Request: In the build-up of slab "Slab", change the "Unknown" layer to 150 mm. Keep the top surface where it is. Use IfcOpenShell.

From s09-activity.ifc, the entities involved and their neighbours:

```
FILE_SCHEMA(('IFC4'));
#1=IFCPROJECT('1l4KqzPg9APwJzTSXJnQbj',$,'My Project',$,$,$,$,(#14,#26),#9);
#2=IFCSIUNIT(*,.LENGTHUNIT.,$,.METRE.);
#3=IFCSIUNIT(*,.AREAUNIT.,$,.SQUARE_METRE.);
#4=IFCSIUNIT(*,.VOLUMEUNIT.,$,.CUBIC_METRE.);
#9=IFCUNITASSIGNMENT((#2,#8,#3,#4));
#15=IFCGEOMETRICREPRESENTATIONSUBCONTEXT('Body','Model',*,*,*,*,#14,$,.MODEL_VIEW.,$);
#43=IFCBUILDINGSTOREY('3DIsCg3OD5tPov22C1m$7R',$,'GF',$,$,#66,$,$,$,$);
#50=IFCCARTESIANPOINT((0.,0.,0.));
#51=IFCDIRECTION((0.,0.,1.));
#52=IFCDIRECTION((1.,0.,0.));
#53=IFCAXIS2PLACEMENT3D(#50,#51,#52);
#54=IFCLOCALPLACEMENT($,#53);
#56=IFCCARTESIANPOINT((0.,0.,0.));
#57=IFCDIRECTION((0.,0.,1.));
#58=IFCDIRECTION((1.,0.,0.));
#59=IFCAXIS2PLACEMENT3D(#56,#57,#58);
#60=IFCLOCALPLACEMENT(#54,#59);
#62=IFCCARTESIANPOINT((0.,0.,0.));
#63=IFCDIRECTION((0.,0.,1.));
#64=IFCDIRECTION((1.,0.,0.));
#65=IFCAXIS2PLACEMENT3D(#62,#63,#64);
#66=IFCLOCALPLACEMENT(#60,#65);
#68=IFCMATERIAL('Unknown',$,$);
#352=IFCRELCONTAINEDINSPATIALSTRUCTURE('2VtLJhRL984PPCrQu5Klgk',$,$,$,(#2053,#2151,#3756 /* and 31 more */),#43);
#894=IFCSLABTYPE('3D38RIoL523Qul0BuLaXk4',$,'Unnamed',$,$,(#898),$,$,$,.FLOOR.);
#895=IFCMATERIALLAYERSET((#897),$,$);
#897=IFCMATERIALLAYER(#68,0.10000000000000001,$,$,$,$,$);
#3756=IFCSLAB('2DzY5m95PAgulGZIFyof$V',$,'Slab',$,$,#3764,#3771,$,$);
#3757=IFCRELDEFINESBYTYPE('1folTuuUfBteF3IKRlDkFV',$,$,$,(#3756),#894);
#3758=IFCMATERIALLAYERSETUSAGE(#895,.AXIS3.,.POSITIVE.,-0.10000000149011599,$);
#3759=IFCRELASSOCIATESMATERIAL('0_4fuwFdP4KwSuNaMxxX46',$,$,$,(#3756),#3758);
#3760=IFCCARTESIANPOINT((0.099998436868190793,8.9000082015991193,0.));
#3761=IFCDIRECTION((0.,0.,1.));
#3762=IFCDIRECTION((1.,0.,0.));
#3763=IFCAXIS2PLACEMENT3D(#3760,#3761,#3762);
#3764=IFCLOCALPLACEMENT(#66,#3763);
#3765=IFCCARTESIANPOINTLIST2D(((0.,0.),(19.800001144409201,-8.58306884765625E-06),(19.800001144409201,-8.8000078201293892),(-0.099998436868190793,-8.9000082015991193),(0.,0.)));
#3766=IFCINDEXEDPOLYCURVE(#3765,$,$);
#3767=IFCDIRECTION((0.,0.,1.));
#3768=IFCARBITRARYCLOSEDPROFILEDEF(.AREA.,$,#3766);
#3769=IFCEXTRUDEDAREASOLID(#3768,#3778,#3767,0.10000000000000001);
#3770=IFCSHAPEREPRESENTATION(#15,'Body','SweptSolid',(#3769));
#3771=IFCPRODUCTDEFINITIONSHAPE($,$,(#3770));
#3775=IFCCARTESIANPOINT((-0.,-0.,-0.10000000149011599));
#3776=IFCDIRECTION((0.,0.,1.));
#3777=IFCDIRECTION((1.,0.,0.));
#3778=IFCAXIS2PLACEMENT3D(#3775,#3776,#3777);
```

```python
import ifcopenshell
import ifcopenshell.util.element
import ifcopenshell.util.representation
import ifcopenshell.util.unit

model = ifcopenshell.open("s09-activity.ifc")
unit_scale = ifcopenshell.util.unit.calculate_unit_scale(model)

layer_set = model.by_id(895)
layer = next(l for l in layer_set.MaterialLayers if l.Material and l.Material.Name == "Unknown")
change = 0.15 / unit_scale - layer.LayerThickness
layer.LayerThickness += change

# Geometry does not follow the layer set by itself.
slabs = [e for e in ifcopenshell.util.element.get_elements_by_material(model, layer_set) if e.is_a("IfcSlab")]
for slab in sorted(slabs, key=lambda e: e.id()):
    body = ifcopenshell.util.representation.get_representation(slab, "Model", "Body")
    solid = body.Items[0]
    old_depth = solid.Depth
    solid.Depth += change
    # Extruded upwards: lower the start of the extrusion so the top stays.
    x, y, z = solid.Position.Location.Coordinates
    solid.Position.Location = model.createIfcCartesianPoint((x, y, z - change))
    print(slab.id(), f"{old_depth:g} -> {solid.Depth:g}")

# The layers are counted up from the underside, which has moved.
for usage in {ifcopenshell.util.element.get_material(slab) for slab in slabs}:
    usage.OffsetFromReferenceLine -= change

model.write("s09-activity_v2.ifc")
```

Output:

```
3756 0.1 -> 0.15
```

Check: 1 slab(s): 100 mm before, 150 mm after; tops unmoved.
